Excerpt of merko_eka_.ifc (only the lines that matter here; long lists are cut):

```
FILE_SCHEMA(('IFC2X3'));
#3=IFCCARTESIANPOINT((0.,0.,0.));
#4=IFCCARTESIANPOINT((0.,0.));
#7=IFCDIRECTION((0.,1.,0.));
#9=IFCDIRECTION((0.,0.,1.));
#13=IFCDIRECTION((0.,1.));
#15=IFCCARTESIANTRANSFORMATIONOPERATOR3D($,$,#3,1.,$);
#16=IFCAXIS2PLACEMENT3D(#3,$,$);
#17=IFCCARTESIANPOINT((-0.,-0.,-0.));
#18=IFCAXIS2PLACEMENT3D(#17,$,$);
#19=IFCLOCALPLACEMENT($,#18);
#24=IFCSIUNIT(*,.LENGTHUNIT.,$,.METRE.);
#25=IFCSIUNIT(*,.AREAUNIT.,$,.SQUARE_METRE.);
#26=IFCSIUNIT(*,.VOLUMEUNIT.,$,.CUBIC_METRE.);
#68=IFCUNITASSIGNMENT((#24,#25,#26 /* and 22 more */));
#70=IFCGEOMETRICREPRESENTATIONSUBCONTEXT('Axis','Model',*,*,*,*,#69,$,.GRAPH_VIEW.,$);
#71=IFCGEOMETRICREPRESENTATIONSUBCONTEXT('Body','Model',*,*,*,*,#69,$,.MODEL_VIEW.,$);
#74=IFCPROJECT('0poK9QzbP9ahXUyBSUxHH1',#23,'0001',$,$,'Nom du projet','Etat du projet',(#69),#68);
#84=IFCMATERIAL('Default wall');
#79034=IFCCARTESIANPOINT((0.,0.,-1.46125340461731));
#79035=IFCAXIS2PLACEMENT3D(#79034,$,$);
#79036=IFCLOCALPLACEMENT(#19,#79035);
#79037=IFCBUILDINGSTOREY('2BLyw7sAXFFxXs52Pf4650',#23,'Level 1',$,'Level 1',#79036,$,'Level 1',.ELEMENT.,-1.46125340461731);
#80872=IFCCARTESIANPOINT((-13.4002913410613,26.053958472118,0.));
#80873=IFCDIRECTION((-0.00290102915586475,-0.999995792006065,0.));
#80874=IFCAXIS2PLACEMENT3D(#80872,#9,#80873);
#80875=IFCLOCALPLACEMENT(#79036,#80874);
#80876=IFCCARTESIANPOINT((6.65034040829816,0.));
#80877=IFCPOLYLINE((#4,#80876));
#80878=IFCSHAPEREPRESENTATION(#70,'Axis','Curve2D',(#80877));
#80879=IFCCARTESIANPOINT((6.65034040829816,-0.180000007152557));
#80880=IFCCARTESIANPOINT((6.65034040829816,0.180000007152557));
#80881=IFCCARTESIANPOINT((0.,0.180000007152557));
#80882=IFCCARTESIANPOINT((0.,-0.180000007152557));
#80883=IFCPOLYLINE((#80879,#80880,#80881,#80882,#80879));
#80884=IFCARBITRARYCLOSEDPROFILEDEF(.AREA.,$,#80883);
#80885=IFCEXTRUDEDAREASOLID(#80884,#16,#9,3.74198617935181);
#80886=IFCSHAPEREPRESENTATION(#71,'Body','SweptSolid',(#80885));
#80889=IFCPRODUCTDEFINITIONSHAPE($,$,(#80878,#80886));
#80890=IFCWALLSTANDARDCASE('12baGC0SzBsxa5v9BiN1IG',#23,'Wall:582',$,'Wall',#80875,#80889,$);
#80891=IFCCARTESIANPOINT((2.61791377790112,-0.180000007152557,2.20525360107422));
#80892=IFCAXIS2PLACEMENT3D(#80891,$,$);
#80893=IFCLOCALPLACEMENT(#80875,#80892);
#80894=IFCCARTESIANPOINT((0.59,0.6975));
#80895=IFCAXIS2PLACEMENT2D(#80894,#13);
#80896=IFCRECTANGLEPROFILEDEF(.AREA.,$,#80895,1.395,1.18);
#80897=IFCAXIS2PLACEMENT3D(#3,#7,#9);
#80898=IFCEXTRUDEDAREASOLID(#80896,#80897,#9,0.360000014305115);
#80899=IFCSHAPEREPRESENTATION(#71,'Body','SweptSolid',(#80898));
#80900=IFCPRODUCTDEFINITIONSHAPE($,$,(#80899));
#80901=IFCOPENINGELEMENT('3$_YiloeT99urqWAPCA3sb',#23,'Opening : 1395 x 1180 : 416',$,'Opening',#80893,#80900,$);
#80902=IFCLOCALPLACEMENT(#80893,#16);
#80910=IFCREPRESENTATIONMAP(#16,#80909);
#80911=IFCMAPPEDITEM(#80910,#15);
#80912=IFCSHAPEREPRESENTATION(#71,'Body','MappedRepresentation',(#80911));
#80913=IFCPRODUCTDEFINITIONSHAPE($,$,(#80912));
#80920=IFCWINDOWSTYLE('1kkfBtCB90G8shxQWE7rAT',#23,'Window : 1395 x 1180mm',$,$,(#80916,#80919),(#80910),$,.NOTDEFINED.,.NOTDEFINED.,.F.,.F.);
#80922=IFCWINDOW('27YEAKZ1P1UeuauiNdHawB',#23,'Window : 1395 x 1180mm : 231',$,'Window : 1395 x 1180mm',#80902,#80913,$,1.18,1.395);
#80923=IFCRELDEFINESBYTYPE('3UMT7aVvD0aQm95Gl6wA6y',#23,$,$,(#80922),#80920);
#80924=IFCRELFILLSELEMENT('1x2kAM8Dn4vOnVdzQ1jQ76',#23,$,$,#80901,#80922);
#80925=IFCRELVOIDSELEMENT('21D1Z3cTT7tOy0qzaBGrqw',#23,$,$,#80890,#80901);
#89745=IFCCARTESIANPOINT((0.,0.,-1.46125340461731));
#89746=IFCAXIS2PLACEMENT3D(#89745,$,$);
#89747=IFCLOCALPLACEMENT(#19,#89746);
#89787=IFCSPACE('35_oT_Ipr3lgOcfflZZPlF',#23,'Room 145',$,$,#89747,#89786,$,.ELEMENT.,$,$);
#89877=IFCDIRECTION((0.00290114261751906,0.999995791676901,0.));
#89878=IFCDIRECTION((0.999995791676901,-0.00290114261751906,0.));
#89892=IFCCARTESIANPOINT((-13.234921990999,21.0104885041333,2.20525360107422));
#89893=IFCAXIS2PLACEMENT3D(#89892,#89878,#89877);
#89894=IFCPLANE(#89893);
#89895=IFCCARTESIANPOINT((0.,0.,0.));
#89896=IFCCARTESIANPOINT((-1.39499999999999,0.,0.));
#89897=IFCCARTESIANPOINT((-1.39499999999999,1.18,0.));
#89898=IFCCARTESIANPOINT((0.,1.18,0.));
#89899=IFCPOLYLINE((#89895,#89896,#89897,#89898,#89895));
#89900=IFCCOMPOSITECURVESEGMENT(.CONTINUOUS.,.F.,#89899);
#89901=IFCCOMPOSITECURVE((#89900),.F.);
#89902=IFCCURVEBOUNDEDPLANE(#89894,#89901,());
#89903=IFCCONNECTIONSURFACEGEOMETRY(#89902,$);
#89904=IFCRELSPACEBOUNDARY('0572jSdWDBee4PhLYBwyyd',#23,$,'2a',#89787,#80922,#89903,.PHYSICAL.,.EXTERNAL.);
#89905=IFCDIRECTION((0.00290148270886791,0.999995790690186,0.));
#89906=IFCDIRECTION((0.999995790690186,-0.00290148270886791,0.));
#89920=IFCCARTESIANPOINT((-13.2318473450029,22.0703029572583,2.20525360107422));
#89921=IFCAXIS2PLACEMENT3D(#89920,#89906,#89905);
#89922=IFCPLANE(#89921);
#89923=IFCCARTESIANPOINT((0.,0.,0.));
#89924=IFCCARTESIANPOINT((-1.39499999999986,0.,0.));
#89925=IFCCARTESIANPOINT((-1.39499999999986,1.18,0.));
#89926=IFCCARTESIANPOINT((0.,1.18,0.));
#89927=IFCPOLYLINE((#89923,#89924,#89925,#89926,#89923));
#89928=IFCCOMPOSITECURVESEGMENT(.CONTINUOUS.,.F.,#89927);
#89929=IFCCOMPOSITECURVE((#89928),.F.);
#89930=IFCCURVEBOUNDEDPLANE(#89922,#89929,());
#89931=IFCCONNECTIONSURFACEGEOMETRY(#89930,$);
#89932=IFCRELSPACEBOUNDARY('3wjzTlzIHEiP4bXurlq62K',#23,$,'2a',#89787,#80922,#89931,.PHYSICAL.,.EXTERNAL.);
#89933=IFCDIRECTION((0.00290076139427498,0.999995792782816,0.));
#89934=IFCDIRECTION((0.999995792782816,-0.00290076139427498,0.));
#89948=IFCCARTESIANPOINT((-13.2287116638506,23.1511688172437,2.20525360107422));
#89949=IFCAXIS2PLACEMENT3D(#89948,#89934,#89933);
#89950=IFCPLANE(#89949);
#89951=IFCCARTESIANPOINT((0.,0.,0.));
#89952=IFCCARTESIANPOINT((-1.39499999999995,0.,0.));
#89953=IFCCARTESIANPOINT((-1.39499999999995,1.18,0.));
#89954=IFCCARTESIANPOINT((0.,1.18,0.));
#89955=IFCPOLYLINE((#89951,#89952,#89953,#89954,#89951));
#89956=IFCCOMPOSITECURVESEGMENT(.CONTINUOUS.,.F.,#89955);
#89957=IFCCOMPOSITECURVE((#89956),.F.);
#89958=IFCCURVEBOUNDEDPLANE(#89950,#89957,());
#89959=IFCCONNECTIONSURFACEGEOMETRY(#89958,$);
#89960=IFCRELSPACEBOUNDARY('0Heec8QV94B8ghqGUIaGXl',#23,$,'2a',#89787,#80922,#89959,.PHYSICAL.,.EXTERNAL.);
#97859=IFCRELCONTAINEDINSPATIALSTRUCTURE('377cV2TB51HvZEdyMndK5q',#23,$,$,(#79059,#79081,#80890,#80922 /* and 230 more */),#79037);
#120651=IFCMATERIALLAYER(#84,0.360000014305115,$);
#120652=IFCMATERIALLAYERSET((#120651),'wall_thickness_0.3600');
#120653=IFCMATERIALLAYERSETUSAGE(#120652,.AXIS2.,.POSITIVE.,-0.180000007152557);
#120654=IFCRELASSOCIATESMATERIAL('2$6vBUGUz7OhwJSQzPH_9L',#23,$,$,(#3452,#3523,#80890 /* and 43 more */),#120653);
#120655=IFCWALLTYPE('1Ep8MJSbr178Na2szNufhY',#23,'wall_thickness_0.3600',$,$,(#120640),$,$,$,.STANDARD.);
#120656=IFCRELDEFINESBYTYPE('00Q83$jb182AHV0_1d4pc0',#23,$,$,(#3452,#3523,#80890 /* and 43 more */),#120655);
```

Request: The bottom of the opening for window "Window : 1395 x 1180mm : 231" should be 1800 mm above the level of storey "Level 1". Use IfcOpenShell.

```python
import numpy as np
import ifcopenshell
import ifcopenshell.api.geometry
import ifcopenshell.geom
import ifcopenshell.util.element
import ifcopenshell.util.placement
import ifcopenshell.util.shape
import ifcopenshell.util.unit

model = ifcopenshell.open("merko_eka_.ifc")
unit_scale = ifcopenshell.util.unit.calculate_unit_scale(model)

window = model.by_guid("27YEAKZ1P1UeuauiNdHawB")
opening = window.FillsVoids[0].RelatingOpeningElement
storey = ifcopenshell.util.element.get_container(window, ifc_class="IfcBuildingStorey")
level = ifcopenshell.util.placement.get_local_placement(storey.ObjectPlacement)[2, 3]

# The opening's origin need not be at the sill, so measure its lowest point.
shape = ifcopenshell.geom.create_shape(ifcopenshell.geom.settings(), opening)
bottom = ifcopenshell.util.shape.get_shape_bottom_elevation(shape, shape.geometry) / unit_scale
dz = level + 1.8 - bottom

shift = np.array([0.0, 0.0, dz])
# The window is placed relative to its opening, so it follows when the opening moves.
matrix = ifcopenshell.util.placement.get_local_placement(opening.ObjectPlacement)
matrix[:3, 3] += shift
ifcopenshell.api.geometry.edit_object_placement(
    model, product=opening, matrix=matrix, is_si=False, should_transform_children=True
)

# Space boundary surfaces are stored in each space's coordinates; move them too.
for rel in window.ProvidesBoundaries:
    if not rel.ConnectionGeometry:
        continue
    surface = rel.ConnectionGeometry.SurfaceOnRelatingElement.BasisSurface
    space_matrix = ifcopenshell.util.placement.get_local_placement(rel.RelatingSpace.ObjectPlacement)
    point = np.array(surface.Position.Location.Coordinates) + space_matrix[:3, :3].T @ shift
    surface.Position = model.createIfcAxis2Placement3D(
        model.createIfcCartesianPoint(point.tolist()), surface.Position.Axis, surface.Position.RefDirection
    )

print(f"moved by {dz * unit_scale:+.3f} m")

model.write("merko_eka__edited.ifc")
```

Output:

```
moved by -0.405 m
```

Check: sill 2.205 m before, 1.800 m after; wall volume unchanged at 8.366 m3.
